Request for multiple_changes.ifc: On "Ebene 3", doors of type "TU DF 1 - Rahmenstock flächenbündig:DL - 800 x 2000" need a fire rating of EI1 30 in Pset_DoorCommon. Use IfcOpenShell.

First a look at what the model holds.

```python
import ifcopenshell
import ifcopenshell.util.element

model = ifcopenshell.open("multiple_changes.ifc")
print(model.schema)
storey = next(s for s in model.by_type("IfcBuildingStorey") if s.Name == "Ebene 3")
doors = [e for e in ifcopenshell.util.element.get_decomposition(storey) if e.is_a("IfcDoor")]
seen = {}
for e in doors:
    element_type = ifcopenshell.util.element.get_type(e)
    key = (element_type.Name if element_type != e and element_type else None, ifcopenshell.util.element.get_pset(e, "Pset_DoorCommon", "FireRating"))
    seen[key] = seen.get(key, 0) + 1
for (name, value), count in sorted(seen.items(), key=str):
    print(count, "x", name, "|", value)
```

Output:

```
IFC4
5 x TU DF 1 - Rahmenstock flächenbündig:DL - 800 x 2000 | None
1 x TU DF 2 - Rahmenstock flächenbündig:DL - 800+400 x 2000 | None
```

```python
import ifcopenshell
import ifcopenshell.api.pset
import ifcopenshell.util.element

model = ifcopenshell.open("multiple_changes.ifc")

storey = next(s for s in model.by_type("IfcBuildingStorey") if s.Name == "Ebene 3")
doors = [e for e in ifcopenshell.util.element.get_decomposition(storey) if e.is_a("IfcDoor")]

count = 0
for e in doors:
    element_type = ifcopenshell.util.element.get_type(e)
    if element_type in (None, e) or element_type.Name != "TU DF 1 - Rahmenstock flächenbündig:DL - 800 x 2000":
        continue
    # add_pset returns the element's existing set when there is one.
    pset = ifcopenshell.api.pset.add_pset(model, product=e, name="Pset_DoorCommon")
    ifcopenshell.api.pset.edit_pset(model, pset=pset, properties={"FireRating": "EI1 30"})
    count += 1

print(count, "doors updated")

model.write("multiple_changes_rev.ifc")
```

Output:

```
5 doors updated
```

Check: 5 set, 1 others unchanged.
